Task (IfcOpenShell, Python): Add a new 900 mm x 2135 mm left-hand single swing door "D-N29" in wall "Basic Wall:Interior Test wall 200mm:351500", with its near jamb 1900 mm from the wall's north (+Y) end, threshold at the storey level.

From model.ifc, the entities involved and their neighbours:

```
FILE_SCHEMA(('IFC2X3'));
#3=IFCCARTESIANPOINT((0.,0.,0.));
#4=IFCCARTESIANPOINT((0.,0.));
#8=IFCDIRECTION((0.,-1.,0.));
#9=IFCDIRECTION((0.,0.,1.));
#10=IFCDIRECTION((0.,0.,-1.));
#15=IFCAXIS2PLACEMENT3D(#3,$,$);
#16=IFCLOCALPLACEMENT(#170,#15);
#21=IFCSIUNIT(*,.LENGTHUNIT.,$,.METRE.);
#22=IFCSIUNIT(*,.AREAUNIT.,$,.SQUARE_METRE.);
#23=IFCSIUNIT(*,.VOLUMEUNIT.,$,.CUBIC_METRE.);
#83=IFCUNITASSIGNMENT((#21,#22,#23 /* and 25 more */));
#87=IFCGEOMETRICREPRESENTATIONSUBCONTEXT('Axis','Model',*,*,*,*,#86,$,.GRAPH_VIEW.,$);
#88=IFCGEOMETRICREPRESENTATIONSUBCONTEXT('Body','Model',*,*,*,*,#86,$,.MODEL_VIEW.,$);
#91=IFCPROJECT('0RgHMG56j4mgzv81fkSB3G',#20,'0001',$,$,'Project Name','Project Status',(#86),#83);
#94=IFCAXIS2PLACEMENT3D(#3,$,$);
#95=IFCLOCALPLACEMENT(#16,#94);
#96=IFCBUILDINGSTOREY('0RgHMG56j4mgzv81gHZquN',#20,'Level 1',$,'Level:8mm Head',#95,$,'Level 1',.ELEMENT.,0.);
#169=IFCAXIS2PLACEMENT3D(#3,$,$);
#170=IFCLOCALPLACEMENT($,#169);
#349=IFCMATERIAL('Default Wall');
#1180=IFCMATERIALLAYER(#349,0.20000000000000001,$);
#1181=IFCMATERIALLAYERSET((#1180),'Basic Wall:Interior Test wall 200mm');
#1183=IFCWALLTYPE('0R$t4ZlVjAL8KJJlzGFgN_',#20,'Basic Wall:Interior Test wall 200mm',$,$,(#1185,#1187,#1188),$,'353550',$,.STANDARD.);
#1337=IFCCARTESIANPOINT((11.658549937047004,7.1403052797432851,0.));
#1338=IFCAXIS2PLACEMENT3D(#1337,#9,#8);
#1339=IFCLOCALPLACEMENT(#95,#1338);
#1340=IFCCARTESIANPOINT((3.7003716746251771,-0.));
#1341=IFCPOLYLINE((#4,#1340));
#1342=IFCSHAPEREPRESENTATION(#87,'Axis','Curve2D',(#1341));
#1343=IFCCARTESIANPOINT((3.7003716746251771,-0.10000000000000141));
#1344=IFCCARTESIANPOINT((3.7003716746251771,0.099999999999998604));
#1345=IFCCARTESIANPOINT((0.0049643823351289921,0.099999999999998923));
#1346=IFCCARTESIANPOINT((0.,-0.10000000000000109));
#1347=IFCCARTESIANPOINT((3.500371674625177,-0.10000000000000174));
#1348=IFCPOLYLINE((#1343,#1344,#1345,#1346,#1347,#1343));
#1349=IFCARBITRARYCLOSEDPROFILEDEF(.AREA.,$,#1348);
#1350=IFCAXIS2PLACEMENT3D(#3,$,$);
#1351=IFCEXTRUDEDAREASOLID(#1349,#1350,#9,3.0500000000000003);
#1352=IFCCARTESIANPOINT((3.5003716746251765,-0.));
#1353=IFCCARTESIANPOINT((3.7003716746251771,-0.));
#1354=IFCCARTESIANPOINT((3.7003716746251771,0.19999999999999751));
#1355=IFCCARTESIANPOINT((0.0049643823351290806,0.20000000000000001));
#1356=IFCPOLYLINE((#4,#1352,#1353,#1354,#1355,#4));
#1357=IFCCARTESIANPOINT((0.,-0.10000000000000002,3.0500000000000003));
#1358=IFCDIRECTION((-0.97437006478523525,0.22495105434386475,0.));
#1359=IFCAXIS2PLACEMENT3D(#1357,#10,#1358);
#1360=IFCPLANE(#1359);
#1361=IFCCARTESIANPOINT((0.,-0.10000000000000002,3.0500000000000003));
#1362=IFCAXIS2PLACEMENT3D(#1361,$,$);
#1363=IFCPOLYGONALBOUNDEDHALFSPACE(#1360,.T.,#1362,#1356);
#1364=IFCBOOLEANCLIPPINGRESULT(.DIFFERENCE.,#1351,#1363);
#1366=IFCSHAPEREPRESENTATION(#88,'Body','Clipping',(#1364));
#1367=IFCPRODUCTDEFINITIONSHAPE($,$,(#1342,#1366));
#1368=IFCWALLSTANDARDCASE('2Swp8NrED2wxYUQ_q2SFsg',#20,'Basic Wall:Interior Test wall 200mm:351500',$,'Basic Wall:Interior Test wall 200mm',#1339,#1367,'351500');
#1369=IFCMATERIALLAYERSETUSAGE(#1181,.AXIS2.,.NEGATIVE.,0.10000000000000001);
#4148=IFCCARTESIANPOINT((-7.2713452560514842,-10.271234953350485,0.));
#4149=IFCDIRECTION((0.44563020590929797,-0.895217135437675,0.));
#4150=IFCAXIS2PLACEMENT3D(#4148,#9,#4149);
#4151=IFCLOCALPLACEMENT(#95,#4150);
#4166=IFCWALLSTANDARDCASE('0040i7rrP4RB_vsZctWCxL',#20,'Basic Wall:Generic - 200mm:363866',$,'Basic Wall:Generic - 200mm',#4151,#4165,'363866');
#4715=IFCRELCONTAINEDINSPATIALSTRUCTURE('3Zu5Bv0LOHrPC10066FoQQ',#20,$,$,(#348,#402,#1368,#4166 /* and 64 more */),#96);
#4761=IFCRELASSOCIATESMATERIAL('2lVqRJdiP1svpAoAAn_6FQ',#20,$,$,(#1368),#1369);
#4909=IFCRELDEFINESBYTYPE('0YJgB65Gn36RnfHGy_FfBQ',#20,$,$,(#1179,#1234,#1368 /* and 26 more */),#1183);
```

```python
import numpy as np
import ifcopenshell
import ifcopenshell.api.feature
import ifcopenshell.api.geometry
import ifcopenshell.api.root
import ifcopenshell.api.spatial
import ifcopenshell.api.type
import ifcopenshell.geom
import ifcopenshell.util.element
import ifcopenshell.util.placement
import ifcopenshell.util.representation
import ifcopenshell.util.shape
import ifcopenshell.util.unit

model = ifcopenshell.open("model.ifc")
unit_scale = ifcopenshell.util.unit.calculate_unit_scale(model)
settings = ifcopenshell.geom.settings()


def volume(element):
    """Net volume in cubic metres, openings subtracted."""
    shape = ifcopenshell.geom.create_shape(settings, element)
    return ifcopenshell.util.shape.get_volume(shape.geometry)


wall = model.by_id(1368)
storey = ifcopenshell.util.element.get_container(wall, ifc_class="IfcBuildingStorey")
context = ifcopenshell.util.representation.get_context(model, "Model", "Body", "MODEL_VIEW")
before = volume(wall)

width, height, from_end, sill = 0.9, 2.135, 1.9, 0.0  # metres

# The wall runs along its own X axis, and the end named is its -X end.
wall_shape = ifcopenshell.geom.create_shape(settings, wall)
x, y, z = ifcopenshell.util.shape.get_vertices(wall_shape.geometry).T
start = x.min() + from_end
face, thickness = float(y.min()), float(y.max() - y.min())
wall_matrix = ifcopenshell.util.placement.get_local_placement(wall.ObjectPlacement)
level = ifcopenshell.util.placement.get_local_placement(storey.ObjectPlacement)[2, 3]


def in_wall(x, y):
    """Placement at x, y metres in the wall's axes, at sill height."""
    matrix = wall_matrix.copy()
    matrix[:, 3] = wall_matrix @ np.array([x / unit_scale, y / unit_scale, 0.0, 1.0])
    matrix[2, 3] = level + sill / unit_scale
    return matrix


# Opening: a box that overshoots both wall faces by 50 mm.
opening = ifcopenshell.api.root.create_entity(model, ifc_class="IfcOpeningElement")
box = ifcopenshell.api.geometry.add_wall_representation(
    model, context=context, length=width, height=height, thickness=thickness + 0.1
)
ifcopenshell.api.geometry.assign_representation(model, product=opening, representation=box)
ifcopenshell.api.geometry.edit_object_placement(model, product=opening, matrix=in_wall(start, face - 0.05), is_si=False)
ifcopenshell.api.feature.add_feature(model, feature=opening, element=wall)

door = ifcopenshell.api.root.create_entity(model, ifc_class="IfcDoor", name="D-N29")
door.OverallWidth, door.OverallHeight = width / unit_scale, height / unit_scale
body = ifcopenshell.api.geometry.add_door_representation(
    model,
    context=context,
    overall_width=door.OverallWidth,
    overall_height=door.OverallHeight,
    operation_type="SINGLE_SWING_LEFT",
    lining_properties={"LiningDepth": thickness / unit_scale, "ThresholdDepth": thickness / unit_scale},
)
ifcopenshell.api.geometry.assign_representation(model, product=door, representation=body)
ifcopenshell.api.spatial.assign_container(model, products=[door], relating_structure=storey)
fills = ifcopenshell.api.feature.add_filling(model, opening=opening, element=door)
fills.OwnerHistory = door.OwnerHistory  # required in IFC2X3

# IFC2X3 keeps the operation on the door style.
style = ifcopenshell.api.root.create_entity(model, ifc_class="IfcDoorStyle", name="D-N29")
style.OperationType, style.ConstructionType = "SINGLE_SWING_LEFT", "NOTDEFINED"
style.ParameterTakesPrecedence = style.Sizeable = False
ifcopenshell.api.type.assign_type(model, related_objects=[door], relating_type=style)

# The lining spans the wall, so the door starts at the wall face.
ifcopenshell.api.geometry.edit_object_placement(model, product=door, matrix=in_wall(start, face), is_si=False)

after = volume(wall)

print(f"wall volume {before:.3f} -> {after:.3f} m3")

model.write("model_rev.ifc")
```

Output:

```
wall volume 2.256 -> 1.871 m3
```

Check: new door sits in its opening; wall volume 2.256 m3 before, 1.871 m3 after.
